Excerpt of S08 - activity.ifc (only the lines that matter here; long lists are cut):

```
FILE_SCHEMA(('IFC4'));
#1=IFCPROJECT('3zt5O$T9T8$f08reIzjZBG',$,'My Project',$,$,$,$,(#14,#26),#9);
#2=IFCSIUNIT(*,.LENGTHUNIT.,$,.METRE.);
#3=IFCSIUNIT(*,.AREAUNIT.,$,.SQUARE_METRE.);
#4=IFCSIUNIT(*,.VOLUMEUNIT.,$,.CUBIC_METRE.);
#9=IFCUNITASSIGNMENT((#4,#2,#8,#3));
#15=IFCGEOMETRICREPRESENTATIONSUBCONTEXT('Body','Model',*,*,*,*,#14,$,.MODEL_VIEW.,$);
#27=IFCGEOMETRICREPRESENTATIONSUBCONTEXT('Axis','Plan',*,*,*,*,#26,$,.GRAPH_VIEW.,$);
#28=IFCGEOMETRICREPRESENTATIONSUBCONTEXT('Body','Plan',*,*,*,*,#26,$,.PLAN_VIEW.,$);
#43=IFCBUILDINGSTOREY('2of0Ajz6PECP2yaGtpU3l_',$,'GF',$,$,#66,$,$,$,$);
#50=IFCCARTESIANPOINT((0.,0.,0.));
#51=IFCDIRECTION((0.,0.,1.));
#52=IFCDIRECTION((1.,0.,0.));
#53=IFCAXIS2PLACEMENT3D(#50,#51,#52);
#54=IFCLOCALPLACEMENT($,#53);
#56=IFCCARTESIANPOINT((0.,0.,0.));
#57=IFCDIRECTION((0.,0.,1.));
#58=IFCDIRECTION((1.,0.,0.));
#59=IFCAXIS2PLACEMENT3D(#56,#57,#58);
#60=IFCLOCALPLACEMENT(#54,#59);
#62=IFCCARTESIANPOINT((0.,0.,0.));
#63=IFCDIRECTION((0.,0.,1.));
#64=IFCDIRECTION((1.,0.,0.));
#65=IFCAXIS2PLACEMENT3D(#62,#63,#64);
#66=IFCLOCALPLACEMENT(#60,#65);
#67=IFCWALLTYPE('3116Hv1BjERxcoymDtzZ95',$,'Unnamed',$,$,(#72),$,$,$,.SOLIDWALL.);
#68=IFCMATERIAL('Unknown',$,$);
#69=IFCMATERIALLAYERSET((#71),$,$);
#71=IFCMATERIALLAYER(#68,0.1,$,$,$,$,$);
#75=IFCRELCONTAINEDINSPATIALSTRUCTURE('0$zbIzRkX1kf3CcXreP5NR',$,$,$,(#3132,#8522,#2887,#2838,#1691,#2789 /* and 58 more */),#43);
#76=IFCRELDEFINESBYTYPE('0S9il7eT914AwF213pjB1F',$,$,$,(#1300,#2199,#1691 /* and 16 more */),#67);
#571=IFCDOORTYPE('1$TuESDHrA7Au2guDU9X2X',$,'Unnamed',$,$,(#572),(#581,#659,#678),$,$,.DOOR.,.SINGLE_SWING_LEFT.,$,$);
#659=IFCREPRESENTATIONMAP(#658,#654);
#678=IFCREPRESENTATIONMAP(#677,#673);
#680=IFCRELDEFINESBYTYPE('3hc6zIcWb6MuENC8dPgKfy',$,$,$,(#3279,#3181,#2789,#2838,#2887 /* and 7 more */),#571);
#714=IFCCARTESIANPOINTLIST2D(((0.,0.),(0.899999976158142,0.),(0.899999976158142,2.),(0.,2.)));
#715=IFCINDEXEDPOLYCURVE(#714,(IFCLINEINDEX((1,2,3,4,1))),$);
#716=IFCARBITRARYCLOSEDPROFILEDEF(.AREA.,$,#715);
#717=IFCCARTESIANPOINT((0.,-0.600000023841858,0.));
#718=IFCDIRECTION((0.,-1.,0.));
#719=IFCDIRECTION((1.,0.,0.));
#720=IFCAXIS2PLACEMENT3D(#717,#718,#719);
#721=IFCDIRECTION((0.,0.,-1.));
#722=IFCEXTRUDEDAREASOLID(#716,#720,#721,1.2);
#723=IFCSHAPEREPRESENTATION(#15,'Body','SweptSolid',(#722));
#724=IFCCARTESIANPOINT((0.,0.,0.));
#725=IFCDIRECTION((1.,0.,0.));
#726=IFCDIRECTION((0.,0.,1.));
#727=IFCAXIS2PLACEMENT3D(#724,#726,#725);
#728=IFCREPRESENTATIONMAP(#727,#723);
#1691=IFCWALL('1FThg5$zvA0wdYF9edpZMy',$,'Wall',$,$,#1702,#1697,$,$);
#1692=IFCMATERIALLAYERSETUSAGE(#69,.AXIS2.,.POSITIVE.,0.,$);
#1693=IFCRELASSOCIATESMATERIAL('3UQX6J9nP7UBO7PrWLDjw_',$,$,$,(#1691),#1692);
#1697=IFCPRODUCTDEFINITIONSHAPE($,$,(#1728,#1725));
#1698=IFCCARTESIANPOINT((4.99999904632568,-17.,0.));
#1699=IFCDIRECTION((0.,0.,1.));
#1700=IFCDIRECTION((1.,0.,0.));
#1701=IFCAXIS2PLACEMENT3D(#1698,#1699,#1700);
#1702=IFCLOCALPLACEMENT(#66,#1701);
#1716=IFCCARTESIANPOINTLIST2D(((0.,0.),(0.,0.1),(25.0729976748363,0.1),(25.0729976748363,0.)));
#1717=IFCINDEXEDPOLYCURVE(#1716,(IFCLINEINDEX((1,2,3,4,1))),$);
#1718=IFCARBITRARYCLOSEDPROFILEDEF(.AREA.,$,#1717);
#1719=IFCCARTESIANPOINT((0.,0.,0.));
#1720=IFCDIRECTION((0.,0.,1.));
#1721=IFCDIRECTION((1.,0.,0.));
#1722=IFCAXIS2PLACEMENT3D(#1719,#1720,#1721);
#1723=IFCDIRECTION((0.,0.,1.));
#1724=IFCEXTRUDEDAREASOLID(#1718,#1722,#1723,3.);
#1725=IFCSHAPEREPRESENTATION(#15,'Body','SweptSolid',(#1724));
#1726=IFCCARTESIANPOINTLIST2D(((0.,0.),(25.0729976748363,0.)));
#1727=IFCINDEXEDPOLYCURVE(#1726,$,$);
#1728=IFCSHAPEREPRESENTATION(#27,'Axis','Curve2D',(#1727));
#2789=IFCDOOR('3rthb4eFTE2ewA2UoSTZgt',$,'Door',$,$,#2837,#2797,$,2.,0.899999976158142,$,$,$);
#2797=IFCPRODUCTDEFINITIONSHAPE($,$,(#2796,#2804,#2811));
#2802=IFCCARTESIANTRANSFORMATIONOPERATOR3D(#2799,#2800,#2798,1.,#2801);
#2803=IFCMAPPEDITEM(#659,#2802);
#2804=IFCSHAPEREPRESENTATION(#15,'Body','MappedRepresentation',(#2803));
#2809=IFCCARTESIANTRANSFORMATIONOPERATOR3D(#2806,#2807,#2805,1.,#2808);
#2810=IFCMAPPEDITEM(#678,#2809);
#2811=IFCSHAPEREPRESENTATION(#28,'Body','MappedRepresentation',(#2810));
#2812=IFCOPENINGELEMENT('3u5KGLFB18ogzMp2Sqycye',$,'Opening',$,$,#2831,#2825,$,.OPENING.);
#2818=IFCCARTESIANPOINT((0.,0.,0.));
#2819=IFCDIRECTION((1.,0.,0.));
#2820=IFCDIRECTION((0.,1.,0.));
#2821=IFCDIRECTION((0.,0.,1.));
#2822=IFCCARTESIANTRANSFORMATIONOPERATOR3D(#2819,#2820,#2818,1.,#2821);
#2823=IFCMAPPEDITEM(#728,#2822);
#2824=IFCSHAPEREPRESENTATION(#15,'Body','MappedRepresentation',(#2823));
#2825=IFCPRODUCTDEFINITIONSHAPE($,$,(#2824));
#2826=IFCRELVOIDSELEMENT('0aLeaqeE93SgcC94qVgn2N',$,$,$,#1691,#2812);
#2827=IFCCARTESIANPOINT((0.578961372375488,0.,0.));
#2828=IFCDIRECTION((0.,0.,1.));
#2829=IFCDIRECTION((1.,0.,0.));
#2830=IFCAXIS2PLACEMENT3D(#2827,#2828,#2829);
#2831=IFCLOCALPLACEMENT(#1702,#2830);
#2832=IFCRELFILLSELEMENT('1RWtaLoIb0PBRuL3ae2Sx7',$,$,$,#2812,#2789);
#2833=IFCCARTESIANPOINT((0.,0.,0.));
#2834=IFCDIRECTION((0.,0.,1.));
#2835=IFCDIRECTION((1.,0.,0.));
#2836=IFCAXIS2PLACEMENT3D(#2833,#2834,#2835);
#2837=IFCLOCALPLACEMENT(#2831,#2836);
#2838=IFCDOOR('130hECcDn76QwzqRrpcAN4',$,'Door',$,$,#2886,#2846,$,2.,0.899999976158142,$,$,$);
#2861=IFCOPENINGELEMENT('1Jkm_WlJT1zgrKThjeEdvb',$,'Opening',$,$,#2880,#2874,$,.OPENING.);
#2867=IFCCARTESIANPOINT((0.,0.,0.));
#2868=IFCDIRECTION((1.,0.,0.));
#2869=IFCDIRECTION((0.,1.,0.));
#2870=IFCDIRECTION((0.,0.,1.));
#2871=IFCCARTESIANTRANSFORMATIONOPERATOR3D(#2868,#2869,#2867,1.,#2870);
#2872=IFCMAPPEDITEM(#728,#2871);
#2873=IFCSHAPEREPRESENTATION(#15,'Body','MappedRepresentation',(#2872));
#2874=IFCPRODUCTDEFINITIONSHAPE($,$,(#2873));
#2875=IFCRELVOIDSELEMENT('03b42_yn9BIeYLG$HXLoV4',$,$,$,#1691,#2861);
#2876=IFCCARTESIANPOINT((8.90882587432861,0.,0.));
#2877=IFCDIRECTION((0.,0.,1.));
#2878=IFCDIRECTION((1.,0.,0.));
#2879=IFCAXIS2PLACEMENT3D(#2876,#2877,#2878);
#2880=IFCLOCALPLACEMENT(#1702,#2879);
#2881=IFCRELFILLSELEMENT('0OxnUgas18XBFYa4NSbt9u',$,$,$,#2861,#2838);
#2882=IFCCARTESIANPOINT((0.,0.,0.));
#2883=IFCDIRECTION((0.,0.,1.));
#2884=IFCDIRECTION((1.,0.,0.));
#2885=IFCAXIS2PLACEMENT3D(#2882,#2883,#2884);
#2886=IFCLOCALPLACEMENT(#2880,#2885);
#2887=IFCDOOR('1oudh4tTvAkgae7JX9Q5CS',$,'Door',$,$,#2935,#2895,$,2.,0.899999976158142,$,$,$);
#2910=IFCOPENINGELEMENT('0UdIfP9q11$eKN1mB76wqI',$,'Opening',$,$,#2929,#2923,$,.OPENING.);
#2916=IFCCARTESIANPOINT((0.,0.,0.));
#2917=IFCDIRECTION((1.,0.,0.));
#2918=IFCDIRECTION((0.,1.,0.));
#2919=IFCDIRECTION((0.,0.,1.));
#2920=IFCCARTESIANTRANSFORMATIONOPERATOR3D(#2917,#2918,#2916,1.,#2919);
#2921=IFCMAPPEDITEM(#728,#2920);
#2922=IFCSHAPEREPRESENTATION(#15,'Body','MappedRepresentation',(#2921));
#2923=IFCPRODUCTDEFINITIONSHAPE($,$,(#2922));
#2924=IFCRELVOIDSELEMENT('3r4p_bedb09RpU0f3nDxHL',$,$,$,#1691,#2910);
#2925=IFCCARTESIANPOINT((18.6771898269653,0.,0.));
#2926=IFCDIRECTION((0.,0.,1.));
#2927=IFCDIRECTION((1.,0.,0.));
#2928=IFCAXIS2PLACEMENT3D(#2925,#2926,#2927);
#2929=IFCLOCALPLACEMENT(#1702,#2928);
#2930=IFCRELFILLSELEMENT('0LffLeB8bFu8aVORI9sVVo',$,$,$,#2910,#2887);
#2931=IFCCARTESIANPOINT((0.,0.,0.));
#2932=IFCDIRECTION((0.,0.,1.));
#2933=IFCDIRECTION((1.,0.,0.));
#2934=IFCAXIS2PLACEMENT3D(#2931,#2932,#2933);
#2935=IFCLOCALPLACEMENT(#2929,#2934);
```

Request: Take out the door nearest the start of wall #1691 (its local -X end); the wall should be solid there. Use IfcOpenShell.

```python
import ifcopenshell
import ifcopenshell.api.feature
import ifcopenshell.api.root
import ifcopenshell.geom
import ifcopenshell.util.shape

model = ifcopenshell.open("S08 - activity.ifc")
settings = ifcopenshell.geom.settings()


def volume(element):
    """Net volume in cubic metres, openings subtracted."""
    shape = ifcopenshell.geom.create_shape(settings, element)
    return ifcopenshell.util.shape.get_volume(shape.geometry)


door = model.by_id(2789)
opening = door.FillsVoids[0].RelatingOpeningElement
wall = opening.VoidsElements[0].RelatingBuildingElement
before = volume(wall)

ifcopenshell.api.root.remove_product(model, product=door)
ifcopenshell.api.feature.remove_feature(model, feature=opening)

after = volume(wall)

print(f"wall volume {before:.3f} -> {after:.3f} m3")

model.write("S08 - activity_rev.ifc")
```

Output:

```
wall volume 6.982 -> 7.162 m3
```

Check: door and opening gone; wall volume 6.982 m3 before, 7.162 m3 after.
